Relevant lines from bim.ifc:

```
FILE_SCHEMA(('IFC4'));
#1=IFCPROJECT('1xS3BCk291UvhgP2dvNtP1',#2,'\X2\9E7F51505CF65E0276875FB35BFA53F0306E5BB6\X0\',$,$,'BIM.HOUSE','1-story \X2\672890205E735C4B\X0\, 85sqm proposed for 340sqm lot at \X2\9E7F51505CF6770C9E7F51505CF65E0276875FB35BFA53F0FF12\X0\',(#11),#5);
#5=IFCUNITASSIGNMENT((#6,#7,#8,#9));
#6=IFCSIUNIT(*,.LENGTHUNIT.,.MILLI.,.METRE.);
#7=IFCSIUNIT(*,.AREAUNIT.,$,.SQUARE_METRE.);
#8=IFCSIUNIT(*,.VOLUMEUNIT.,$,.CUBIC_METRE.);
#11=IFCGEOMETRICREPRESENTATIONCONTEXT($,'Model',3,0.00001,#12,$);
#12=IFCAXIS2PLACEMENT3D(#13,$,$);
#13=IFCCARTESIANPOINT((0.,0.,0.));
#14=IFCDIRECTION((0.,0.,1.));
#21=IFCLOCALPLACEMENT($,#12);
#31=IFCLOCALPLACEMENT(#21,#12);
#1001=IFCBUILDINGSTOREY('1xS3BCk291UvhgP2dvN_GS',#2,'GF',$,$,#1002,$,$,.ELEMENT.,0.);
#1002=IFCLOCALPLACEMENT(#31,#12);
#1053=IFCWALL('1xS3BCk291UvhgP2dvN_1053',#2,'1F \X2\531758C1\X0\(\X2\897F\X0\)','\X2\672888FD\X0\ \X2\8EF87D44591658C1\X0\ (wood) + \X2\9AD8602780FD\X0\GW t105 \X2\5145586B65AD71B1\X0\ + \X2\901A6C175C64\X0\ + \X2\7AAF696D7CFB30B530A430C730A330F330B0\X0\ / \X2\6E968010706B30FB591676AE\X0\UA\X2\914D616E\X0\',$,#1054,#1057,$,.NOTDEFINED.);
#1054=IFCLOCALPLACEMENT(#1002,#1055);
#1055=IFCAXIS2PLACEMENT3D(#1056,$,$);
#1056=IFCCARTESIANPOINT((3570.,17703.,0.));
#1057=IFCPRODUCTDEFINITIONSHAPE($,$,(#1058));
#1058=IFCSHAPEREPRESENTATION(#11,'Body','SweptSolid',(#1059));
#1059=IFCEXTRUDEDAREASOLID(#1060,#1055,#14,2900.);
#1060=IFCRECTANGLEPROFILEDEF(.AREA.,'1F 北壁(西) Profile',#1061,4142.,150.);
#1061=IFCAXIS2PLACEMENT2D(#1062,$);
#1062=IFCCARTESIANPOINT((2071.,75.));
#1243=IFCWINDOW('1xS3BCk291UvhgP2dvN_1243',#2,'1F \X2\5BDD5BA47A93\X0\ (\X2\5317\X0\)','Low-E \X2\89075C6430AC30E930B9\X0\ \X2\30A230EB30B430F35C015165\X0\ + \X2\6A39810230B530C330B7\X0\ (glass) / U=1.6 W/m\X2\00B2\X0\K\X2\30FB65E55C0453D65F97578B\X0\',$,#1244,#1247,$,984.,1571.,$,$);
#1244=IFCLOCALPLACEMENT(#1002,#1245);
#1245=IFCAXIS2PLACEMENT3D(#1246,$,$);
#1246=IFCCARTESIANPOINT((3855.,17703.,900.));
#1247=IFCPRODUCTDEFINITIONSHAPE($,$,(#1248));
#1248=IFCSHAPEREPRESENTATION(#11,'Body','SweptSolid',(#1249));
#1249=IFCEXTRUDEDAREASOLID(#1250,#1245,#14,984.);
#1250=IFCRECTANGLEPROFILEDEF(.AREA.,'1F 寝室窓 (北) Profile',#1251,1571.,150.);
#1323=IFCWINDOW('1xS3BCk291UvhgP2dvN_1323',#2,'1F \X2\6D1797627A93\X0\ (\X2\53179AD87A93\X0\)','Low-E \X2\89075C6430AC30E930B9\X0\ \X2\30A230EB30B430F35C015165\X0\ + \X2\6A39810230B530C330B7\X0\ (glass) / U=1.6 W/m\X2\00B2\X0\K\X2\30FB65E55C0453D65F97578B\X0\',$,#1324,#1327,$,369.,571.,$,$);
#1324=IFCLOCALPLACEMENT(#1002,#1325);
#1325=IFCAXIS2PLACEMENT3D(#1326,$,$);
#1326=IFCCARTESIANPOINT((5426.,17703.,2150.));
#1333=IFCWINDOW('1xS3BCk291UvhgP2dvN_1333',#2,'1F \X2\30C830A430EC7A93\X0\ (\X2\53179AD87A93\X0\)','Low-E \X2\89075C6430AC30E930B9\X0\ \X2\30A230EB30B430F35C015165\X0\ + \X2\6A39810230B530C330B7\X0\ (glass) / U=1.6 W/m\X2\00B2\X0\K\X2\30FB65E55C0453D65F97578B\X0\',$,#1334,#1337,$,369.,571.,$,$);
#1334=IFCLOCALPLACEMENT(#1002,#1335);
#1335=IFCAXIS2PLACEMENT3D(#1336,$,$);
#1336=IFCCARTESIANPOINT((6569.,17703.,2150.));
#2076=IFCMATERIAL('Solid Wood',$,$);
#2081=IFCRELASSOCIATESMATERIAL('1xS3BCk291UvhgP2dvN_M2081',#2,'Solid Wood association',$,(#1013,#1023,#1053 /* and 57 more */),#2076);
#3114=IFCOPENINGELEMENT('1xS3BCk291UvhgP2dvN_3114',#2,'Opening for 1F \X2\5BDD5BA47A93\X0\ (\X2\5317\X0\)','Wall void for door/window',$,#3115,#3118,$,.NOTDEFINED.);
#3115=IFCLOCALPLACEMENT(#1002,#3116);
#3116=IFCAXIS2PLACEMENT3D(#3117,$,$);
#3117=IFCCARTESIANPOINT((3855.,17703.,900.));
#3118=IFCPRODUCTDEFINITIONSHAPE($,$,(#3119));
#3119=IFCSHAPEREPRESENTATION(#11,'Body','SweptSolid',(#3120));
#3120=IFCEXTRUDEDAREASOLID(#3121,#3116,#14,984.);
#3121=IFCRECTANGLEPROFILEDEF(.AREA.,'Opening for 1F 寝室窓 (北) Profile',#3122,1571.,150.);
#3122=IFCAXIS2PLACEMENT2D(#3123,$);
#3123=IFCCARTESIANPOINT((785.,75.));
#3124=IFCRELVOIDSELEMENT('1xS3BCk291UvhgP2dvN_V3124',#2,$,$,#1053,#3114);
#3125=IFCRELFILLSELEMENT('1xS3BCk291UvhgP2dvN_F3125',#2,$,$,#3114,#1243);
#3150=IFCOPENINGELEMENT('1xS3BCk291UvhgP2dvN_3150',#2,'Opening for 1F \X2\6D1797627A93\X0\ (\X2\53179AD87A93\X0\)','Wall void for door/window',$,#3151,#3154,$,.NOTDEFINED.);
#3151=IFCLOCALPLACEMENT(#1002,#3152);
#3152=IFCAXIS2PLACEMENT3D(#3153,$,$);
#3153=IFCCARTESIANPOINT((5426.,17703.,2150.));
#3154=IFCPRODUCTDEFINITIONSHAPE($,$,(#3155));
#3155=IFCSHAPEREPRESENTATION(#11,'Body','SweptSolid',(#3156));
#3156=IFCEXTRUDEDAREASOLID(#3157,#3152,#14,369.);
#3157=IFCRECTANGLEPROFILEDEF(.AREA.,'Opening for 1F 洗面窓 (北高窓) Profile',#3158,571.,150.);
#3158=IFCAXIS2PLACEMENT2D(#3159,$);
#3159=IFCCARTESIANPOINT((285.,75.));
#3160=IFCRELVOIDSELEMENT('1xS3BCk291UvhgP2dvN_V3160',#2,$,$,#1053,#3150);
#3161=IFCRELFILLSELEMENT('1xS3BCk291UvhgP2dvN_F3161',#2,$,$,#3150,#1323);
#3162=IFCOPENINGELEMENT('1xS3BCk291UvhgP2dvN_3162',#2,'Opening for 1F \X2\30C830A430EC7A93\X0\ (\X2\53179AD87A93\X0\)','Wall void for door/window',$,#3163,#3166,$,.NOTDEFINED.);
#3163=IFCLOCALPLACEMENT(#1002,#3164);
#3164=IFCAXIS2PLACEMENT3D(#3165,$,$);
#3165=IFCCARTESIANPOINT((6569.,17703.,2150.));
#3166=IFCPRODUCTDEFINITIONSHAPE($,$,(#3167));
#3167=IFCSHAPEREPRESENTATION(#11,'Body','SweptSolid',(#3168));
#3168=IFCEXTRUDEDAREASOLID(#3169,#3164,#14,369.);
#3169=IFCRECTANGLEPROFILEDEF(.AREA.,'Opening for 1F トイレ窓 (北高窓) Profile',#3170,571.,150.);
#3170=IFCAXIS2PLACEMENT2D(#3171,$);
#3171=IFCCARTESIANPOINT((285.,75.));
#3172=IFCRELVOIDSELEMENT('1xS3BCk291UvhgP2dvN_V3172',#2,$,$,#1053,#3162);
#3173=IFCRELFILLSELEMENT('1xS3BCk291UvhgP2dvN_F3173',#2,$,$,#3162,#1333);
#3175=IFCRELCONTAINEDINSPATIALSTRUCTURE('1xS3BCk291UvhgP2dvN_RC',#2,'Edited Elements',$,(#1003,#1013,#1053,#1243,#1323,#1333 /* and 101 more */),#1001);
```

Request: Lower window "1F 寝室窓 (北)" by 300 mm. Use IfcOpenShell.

```python
import numpy as np
import ifcopenshell
import ifcopenshell.api.geometry
import ifcopenshell.util.placement
import ifcopenshell.util.unit

model = ifcopenshell.open("bim.ifc")
unit_scale = ifcopenshell.util.unit.calculate_unit_scale(model)

window = model.by_guid("1xS3BCk291UvhgP2dvN_1243")
opening = window.FillsVoids[0].RelatingOpeningElement
dz = -300.0

shift = np.array([0.0, 0.0, dz])
# The window is not placed relative to its opening, so move both.
for product in (opening, window):
    matrix = ifcopenshell.util.placement.get_local_placement(product.ObjectPlacement)
    matrix[:3, 3] += shift
    ifcopenshell.api.geometry.edit_object_placement(model, product=product, matrix=matrix, is_si=False)

print(f"moved by {dz * unit_scale:+.3f} m")

model.write("bim_edited.ifc")
```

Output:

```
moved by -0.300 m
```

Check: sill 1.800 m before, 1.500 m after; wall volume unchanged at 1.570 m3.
